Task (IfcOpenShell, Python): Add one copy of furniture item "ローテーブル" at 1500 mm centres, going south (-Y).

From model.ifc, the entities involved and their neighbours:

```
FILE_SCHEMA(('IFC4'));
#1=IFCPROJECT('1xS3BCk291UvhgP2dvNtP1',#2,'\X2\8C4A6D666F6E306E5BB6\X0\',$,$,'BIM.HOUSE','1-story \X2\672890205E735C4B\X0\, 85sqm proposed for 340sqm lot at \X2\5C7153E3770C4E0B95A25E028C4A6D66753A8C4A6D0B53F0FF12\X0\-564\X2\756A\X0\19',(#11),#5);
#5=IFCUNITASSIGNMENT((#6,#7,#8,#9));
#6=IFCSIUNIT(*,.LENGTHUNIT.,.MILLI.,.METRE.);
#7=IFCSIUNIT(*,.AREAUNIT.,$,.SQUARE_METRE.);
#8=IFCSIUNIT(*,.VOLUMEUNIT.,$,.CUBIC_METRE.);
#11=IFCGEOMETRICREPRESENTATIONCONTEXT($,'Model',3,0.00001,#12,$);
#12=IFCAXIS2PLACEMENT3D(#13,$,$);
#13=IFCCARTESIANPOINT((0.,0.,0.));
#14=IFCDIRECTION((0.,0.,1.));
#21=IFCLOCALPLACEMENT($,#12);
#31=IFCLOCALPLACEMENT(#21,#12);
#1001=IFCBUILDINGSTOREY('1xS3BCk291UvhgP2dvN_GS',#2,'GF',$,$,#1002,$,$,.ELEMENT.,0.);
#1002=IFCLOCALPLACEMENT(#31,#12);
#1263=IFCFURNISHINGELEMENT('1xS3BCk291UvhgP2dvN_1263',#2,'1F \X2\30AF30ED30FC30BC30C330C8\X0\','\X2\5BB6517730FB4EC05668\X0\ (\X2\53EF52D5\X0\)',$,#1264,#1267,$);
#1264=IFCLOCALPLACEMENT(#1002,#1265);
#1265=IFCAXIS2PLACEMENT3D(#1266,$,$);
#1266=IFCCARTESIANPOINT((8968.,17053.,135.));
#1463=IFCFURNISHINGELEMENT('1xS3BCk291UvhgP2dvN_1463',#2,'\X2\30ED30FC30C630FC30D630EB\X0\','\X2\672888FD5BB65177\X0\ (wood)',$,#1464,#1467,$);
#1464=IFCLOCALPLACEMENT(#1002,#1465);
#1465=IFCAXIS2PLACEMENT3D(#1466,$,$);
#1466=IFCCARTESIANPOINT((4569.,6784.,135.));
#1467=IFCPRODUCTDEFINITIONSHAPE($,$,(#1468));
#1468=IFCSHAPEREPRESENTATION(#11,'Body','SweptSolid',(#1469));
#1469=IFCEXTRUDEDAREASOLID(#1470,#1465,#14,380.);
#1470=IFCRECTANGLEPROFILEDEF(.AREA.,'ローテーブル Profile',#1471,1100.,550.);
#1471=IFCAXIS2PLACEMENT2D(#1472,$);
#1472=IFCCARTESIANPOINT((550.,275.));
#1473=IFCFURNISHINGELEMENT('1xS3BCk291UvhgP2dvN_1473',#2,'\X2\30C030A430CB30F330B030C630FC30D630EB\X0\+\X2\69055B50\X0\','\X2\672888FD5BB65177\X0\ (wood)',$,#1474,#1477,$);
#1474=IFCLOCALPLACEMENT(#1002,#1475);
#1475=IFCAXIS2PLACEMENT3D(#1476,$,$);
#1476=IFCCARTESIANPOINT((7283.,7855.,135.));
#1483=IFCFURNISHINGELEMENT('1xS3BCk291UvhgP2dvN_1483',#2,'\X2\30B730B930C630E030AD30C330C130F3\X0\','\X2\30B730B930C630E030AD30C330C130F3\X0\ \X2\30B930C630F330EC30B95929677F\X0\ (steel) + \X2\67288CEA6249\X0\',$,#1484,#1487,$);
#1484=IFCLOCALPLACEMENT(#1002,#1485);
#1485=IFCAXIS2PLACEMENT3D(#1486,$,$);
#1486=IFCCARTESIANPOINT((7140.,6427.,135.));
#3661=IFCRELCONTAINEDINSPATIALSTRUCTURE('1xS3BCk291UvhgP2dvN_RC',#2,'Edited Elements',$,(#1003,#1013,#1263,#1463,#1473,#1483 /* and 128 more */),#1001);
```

```python
import numpy as np
import ifcopenshell
import ifcopenshell.api.geometry
import ifcopenshell.api.root
import ifcopenshell.util.element
import ifcopenshell.util.placement

model = ifcopenshell.open("model.ifc")


def reuse_history(source, copy):
    """copy_class also copies each property set's owner history, people and application; keep the originals."""
    for rel in copy.IsDefinedBy:
        if rel.is_a("IfcRelDefinesByProperties") and (history := rel.RelatingPropertyDefinition.OwnerHistory):
            rel.RelatingPropertyDefinition.OwnerHistory = source.OwnerHistory
            ifcopenshell.util.element.remove_deep2(model, history)


source = model.by_id(1463)
base = ifcopenshell.util.placement.get_local_placement(source.ObjectPlacement)
step = np.array([0.0, -1.0, 0.0]) * 1500.0

for i in range(1, 2):
    copy = ifcopenshell.api.root.copy_class(model, product=source)
    copy.Representation = ifcopenshell.util.element.copy_deep(
        model, source.Representation, exclude=["IfcGeometricRepresentationContext", "IfcRepresentationMap"]
    )
    reuse_history(source, copy)
    matrix = base.copy()
    matrix[:3, 3] += i * step
    print("added at", matrix[:3, 3].round(3) + 0.0)
    ifcopenshell.api.geometry.edit_object_placement(model, product=copy, matrix=matrix, is_si=False)

model.write("model_rev.ifc")
```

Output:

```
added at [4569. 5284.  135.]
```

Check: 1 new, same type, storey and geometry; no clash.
